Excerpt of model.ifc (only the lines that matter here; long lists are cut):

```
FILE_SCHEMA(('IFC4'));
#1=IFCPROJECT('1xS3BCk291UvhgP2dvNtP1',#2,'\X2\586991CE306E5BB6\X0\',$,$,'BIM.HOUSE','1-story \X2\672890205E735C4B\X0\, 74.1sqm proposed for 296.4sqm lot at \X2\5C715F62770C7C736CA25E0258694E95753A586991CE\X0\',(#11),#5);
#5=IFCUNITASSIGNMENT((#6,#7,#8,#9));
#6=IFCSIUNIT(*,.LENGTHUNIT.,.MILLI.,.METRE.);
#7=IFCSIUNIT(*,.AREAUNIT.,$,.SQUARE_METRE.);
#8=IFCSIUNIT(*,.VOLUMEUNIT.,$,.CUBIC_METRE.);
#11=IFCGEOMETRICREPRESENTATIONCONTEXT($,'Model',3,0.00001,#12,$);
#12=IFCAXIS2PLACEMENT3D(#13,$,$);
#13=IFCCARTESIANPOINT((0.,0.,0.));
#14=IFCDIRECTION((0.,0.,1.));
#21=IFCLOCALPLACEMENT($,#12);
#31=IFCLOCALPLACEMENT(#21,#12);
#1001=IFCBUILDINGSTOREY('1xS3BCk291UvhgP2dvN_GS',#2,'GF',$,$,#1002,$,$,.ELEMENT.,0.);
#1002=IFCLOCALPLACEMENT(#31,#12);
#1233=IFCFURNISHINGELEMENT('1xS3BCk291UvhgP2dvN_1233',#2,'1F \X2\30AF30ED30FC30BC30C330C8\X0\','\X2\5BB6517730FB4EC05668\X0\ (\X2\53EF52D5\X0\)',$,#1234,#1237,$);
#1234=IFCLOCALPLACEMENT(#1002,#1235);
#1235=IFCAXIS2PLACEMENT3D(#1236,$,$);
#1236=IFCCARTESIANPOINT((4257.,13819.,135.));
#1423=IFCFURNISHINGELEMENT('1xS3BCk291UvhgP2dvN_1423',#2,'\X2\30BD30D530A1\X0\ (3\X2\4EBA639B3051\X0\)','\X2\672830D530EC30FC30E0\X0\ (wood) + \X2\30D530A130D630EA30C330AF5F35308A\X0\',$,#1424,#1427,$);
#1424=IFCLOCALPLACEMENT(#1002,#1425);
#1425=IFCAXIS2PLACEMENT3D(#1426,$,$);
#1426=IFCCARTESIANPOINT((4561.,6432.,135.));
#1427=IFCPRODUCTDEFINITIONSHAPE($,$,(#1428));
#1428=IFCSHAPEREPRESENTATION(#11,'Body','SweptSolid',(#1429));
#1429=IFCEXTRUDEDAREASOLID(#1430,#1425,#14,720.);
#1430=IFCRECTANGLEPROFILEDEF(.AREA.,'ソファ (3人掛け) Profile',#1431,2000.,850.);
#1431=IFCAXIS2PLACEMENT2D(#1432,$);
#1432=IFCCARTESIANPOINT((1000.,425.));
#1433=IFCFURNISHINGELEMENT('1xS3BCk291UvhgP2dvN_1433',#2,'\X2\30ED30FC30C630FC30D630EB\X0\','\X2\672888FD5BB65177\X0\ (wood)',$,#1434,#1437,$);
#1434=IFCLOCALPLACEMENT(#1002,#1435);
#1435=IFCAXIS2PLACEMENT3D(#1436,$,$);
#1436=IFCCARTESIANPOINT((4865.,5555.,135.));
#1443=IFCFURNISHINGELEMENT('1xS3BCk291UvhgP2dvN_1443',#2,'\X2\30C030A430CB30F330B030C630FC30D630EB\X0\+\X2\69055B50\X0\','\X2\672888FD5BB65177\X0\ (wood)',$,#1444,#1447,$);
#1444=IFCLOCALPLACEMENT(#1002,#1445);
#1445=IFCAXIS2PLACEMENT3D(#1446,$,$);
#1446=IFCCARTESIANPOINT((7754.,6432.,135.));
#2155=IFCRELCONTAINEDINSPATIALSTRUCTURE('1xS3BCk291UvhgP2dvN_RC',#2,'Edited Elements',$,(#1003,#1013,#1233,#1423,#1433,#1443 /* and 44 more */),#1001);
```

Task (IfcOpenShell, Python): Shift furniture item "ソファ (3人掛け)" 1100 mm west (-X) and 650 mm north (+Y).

```python
import ifcopenshell
import ifcopenshell.api.geometry
import ifcopenshell.util.placement
import ifcopenshell.util.unit

model = ifcopenshell.open("model.ifc")
unit_scale = ifcopenshell.util.unit.calculate_unit_scale(model)

item = model.by_id(1423)
matrix = ifcopenshell.util.placement.get_local_placement(item.ObjectPlacement)
matrix[0, 3] -= 1.1 / unit_scale
matrix[1, 3] += 0.65 / unit_scale
ifcopenshell.api.geometry.edit_object_placement(model, product=item, matrix=matrix, is_si=False)

print(ifcopenshell.util.placement.get_local_placement(item.ObjectPlacement).round(3) + 0.0)

model.write("model_rev.ifc")
```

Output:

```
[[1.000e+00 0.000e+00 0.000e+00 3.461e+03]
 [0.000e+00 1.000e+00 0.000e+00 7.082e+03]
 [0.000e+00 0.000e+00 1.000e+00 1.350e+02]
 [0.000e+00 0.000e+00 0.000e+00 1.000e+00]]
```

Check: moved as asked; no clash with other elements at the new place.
